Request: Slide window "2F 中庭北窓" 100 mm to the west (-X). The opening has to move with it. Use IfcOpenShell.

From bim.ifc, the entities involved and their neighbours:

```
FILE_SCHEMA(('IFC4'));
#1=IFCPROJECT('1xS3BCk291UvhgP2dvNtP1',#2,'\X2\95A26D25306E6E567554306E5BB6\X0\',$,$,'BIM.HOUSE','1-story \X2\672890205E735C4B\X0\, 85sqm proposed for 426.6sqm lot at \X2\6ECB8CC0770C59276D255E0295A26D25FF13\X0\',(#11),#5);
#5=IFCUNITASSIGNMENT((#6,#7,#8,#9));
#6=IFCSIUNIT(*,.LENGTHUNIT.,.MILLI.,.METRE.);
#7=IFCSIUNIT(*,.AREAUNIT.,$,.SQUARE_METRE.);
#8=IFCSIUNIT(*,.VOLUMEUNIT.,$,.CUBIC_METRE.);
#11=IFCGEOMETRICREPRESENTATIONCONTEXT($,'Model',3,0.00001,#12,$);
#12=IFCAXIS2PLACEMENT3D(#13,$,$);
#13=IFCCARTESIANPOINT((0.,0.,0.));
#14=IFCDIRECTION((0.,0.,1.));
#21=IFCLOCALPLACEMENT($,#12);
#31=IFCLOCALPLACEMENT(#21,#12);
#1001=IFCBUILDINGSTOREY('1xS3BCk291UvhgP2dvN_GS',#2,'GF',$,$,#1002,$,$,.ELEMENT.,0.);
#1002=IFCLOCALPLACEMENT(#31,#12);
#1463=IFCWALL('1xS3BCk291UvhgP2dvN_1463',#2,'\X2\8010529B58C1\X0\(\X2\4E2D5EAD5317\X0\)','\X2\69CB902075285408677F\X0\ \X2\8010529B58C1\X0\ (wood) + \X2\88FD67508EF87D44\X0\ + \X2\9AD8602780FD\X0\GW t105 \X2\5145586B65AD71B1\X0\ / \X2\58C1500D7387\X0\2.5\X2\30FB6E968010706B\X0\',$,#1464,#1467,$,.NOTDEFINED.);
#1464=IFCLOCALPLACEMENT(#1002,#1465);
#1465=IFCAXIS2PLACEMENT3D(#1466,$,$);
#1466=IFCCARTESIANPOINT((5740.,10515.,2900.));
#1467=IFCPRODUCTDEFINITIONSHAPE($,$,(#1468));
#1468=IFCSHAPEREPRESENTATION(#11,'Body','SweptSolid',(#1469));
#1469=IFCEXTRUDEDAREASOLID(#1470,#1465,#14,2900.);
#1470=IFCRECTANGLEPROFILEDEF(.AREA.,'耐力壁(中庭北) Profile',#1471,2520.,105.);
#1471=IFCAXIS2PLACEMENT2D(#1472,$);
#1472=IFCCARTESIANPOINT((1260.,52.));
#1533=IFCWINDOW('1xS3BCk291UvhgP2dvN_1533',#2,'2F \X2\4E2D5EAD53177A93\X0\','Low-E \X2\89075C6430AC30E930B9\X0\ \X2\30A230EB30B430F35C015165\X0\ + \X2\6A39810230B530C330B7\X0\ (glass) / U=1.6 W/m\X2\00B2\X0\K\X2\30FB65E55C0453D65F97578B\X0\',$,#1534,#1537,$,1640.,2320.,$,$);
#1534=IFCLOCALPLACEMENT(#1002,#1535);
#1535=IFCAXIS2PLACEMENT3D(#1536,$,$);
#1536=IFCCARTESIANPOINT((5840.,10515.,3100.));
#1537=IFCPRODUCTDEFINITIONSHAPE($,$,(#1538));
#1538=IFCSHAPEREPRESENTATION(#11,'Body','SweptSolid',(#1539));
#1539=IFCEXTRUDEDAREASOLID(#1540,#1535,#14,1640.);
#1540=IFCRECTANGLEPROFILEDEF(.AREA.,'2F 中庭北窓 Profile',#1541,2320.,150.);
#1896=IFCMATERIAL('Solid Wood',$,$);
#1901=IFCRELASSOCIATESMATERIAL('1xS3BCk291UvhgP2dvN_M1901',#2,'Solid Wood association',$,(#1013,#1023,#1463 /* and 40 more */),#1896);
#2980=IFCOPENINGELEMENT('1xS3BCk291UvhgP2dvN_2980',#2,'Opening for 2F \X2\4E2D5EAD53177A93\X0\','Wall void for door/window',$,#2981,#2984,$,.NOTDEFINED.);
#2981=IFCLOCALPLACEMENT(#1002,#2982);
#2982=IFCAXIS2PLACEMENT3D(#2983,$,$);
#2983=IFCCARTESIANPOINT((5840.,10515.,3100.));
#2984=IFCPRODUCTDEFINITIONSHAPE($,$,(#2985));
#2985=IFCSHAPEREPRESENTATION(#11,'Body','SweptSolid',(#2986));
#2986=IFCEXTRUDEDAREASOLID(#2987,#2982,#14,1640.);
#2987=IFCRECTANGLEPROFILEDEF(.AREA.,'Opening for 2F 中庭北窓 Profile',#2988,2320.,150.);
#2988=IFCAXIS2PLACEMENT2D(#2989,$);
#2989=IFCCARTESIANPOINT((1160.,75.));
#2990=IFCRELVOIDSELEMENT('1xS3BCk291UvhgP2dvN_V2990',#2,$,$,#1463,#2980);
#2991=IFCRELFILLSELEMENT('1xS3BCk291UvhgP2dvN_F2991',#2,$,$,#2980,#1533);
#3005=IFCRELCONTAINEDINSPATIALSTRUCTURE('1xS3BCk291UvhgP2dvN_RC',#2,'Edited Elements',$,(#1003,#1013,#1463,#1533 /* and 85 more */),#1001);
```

```python
import ifcopenshell
import ifcopenshell.api.geometry
import ifcopenshell.util.placement
import ifcopenshell.util.unit

model = ifcopenshell.open("bim.ifc")
unit_scale = ifcopenshell.util.unit.calculate_unit_scale(model)

window = model.by_guid("1xS3BCk291UvhgP2dvN_1533")
opening = window.FillsVoids[0].RelatingOpeningElement
wall = opening.VoidsElements[0].RelatingBuildingElement

wall_matrix = ifcopenshell.util.placement.get_local_placement(wall.ObjectPlacement)
shift = wall_matrix[:3, 0] * -0.1 / unit_scale
before = ifcopenshell.util.placement.get_local_placement(window.ObjectPlacement)[:3, 3].copy()

# The window is not placed relative to its opening, so move both.
for product in (opening, window):
    matrix = ifcopenshell.util.placement.get_local_placement(product.ObjectPlacement)
    matrix[:3, 3] += shift
    ifcopenshell.api.geometry.edit_object_placement(model, product=product, matrix=matrix, is_si=False)

after = ifcopenshell.util.placement.get_local_placement(window.ObjectPlacement)[:3, 3]
print("window moved by", (after - before).round(3) + 0.0)

model.write("bim_v2.ifc")
```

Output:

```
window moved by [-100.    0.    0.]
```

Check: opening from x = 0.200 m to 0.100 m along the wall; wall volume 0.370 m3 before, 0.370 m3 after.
